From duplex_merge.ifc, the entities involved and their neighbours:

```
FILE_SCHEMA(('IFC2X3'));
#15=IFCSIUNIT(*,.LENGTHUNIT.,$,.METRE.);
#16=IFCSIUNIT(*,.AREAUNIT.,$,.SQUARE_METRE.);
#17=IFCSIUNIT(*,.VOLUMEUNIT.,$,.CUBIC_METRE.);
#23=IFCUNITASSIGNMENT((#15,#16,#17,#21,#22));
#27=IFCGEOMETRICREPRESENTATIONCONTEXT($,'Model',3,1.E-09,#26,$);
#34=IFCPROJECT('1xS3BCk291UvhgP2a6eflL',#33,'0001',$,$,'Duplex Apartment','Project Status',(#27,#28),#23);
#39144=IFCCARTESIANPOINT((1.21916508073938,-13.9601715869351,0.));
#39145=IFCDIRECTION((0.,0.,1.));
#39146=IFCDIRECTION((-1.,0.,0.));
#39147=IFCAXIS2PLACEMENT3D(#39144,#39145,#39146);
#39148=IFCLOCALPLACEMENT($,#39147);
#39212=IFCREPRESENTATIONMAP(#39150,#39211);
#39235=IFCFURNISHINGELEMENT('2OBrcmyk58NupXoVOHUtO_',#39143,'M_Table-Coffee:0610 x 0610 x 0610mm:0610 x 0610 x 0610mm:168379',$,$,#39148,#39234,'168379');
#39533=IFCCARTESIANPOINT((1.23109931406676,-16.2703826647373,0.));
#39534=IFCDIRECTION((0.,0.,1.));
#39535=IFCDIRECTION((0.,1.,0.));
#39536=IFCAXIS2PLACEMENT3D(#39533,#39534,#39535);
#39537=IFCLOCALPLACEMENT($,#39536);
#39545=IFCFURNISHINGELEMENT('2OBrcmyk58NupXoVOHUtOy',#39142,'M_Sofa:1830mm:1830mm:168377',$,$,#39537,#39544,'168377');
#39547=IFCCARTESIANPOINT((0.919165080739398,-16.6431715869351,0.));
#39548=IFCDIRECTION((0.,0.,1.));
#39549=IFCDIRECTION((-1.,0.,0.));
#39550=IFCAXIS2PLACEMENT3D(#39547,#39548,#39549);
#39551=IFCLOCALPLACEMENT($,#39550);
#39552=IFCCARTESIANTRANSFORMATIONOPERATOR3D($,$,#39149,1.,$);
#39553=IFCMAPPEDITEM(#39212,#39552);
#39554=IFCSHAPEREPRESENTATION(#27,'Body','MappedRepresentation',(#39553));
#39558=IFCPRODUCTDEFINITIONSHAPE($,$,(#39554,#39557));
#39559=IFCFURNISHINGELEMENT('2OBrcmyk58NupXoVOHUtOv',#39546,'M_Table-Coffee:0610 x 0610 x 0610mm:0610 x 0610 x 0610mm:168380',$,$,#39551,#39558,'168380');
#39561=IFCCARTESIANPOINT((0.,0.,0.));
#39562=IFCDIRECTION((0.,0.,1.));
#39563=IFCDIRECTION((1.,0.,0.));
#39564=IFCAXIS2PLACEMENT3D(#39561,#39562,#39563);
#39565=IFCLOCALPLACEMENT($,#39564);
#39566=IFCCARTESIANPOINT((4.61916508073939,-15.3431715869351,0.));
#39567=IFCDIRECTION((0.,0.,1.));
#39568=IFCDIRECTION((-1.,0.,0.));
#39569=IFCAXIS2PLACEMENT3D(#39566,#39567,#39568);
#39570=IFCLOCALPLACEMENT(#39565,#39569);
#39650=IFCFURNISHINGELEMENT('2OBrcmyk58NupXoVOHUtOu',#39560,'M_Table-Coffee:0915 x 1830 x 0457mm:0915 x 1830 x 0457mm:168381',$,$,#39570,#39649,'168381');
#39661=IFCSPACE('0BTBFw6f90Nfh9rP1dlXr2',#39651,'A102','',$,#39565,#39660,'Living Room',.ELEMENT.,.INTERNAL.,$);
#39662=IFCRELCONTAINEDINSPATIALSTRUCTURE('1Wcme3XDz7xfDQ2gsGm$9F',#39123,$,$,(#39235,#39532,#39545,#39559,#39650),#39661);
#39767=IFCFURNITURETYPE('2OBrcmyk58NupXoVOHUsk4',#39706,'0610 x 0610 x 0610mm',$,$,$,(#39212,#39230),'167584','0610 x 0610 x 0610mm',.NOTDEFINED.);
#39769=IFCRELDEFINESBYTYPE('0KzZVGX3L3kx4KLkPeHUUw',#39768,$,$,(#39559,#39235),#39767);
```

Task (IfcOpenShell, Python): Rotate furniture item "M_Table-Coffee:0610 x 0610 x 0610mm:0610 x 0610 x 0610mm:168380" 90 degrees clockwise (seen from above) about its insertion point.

```python
import ifcopenshell
import ifcopenshell.api.geometry
import ifcopenshell.util.placement

model = ifcopenshell.open("duplex_merge.ifc")

item = model.by_id(39559)
matrix = ifcopenshell.util.placement.get_local_placement(item.ObjectPlacement)
matrix = matrix @ ifcopenshell.util.placement.rotation(-90, "Z")
ifcopenshell.api.geometry.edit_object_placement(model, product=item, matrix=matrix, is_si=False)

print(ifcopenshell.util.placement.get_local_placement(item.ObjectPlacement).round(3) + 0.0)

model.write("duplex_merge-out.ifc")
```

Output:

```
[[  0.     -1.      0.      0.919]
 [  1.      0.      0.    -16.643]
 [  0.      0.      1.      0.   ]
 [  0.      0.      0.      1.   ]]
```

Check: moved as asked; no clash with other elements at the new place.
